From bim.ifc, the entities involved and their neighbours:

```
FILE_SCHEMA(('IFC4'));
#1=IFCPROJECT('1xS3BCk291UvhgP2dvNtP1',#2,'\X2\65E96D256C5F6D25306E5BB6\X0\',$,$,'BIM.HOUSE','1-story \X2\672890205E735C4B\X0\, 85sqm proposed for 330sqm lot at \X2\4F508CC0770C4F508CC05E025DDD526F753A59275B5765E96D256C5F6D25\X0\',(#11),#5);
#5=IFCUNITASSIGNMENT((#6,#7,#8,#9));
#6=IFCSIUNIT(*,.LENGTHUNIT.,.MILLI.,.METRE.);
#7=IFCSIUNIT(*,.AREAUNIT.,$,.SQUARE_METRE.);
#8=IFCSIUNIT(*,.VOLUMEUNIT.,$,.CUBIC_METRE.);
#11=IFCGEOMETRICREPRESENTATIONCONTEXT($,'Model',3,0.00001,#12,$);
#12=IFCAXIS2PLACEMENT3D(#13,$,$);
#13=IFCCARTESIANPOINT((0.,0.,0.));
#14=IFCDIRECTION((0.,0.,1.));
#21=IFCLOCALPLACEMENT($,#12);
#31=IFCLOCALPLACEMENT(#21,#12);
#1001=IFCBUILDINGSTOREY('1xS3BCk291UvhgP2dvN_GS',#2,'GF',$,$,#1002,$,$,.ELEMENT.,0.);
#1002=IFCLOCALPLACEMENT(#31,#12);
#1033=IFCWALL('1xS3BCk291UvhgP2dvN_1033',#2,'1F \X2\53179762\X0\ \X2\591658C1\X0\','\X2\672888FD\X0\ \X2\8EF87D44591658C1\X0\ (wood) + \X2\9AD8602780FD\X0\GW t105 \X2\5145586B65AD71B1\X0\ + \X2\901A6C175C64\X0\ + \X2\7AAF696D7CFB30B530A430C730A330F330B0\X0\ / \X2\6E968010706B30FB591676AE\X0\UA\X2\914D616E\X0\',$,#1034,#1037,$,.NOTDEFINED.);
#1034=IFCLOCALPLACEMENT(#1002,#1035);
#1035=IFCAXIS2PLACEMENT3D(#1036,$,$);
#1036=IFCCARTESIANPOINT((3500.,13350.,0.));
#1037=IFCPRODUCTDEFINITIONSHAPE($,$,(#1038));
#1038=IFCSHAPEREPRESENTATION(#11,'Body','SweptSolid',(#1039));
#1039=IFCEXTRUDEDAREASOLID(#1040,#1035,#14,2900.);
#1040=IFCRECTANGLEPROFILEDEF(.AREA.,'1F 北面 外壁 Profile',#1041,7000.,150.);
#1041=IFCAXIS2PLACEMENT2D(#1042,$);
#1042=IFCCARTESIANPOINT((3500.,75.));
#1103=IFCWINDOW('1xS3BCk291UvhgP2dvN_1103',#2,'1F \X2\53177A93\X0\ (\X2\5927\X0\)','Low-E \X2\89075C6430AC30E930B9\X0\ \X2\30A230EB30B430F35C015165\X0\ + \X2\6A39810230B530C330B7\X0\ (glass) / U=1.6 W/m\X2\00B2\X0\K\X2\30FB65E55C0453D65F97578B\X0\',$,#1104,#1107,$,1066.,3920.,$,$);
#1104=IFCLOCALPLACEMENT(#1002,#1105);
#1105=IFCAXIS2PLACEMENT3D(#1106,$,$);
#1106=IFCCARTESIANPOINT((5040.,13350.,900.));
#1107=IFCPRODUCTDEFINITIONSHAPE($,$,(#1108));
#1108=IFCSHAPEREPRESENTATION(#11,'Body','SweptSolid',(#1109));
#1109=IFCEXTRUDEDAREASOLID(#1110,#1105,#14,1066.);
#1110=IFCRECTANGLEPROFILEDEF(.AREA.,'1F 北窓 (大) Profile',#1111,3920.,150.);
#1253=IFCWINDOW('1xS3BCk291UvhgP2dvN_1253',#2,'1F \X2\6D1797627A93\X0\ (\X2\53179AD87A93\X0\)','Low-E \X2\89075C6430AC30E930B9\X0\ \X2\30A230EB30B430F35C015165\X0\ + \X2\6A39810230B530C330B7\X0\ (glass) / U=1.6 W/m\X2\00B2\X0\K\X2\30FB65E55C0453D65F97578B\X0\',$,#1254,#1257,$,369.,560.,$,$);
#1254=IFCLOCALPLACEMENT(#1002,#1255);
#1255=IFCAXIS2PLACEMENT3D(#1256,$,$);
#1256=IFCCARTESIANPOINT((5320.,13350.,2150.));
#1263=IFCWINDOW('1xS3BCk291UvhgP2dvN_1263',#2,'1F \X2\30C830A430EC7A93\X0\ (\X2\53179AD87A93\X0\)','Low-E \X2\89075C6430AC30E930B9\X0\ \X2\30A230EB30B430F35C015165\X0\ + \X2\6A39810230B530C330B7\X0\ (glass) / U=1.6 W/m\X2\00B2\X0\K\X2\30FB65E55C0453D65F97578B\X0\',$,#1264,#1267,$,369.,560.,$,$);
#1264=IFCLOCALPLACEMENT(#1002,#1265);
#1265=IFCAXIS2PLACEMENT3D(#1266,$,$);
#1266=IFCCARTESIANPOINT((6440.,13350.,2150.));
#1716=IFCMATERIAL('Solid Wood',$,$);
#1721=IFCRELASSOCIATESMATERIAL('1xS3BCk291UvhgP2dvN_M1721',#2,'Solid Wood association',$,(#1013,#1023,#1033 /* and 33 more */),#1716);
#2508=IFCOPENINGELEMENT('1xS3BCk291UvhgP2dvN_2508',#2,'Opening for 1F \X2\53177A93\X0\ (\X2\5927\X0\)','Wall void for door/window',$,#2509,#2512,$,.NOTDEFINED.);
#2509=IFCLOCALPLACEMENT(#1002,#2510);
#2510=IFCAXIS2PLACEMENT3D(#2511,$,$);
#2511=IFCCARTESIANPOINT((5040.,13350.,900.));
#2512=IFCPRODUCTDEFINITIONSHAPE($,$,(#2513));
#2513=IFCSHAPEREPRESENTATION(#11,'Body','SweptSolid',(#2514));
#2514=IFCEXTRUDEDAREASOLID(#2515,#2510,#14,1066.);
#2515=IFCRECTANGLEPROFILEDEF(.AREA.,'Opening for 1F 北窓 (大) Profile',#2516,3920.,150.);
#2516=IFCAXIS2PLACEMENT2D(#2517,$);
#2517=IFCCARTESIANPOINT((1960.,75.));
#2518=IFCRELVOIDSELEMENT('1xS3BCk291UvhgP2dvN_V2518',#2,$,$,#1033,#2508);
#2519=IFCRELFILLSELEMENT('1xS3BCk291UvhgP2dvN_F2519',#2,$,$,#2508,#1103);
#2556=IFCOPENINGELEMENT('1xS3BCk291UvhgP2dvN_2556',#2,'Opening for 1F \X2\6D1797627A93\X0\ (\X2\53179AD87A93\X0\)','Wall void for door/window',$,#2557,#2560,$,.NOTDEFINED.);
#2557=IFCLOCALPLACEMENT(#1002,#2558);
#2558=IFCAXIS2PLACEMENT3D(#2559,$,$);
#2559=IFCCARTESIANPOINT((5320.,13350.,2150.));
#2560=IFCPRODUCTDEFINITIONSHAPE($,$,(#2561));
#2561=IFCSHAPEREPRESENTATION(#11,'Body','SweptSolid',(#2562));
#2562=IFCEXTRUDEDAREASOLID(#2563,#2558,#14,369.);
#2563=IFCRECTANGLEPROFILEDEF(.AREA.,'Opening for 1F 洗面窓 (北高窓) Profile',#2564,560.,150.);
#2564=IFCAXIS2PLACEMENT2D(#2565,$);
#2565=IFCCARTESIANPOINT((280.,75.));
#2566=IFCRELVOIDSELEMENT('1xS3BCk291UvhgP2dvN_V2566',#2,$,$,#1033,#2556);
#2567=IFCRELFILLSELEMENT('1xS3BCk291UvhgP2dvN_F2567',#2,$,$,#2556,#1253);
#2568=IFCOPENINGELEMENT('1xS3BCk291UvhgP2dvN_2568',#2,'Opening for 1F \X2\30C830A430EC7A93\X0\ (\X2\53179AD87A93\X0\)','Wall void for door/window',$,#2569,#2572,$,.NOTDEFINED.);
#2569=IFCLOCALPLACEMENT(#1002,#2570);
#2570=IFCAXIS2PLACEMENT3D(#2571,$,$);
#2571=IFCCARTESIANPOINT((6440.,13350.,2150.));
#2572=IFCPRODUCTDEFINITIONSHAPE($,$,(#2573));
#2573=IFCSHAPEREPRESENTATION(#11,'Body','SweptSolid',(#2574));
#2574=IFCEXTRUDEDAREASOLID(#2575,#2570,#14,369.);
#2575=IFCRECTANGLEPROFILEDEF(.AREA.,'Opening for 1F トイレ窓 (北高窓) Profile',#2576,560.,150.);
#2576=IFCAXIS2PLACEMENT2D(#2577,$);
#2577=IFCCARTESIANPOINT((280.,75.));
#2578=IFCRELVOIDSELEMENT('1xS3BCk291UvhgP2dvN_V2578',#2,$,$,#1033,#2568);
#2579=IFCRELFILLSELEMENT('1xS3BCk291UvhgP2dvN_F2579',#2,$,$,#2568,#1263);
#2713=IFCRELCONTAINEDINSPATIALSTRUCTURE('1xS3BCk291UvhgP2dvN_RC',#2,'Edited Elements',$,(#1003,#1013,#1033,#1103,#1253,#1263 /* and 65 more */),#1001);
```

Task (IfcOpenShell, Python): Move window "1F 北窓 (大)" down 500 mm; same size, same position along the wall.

```python
import numpy as np
import ifcopenshell
import ifcopenshell.api.geometry
import ifcopenshell.util.placement
import ifcopenshell.util.unit

model = ifcopenshell.open("bim.ifc")
unit_scale = ifcopenshell.util.unit.calculate_unit_scale(model)

window = model.by_guid("1xS3BCk291UvhgP2dvN_1103")
opening = window.FillsVoids[0].RelatingOpeningElement
dz = -500.0

shift = np.array([0.0, 0.0, dz])
# The window is not placed relative to its opening, so move both.
for product in (opening, window):
    matrix = ifcopenshell.util.placement.get_local_placement(product.ObjectPlacement)
    matrix[:3, 3] += shift
    ifcopenshell.api.geometry.edit_object_placement(model, product=product, matrix=matrix, is_si=False)

print(f"moved by {dz * unit_scale:+.3f} m")

model.write("bim_v2.ifc")
```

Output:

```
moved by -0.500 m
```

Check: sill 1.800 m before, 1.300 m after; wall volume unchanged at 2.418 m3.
